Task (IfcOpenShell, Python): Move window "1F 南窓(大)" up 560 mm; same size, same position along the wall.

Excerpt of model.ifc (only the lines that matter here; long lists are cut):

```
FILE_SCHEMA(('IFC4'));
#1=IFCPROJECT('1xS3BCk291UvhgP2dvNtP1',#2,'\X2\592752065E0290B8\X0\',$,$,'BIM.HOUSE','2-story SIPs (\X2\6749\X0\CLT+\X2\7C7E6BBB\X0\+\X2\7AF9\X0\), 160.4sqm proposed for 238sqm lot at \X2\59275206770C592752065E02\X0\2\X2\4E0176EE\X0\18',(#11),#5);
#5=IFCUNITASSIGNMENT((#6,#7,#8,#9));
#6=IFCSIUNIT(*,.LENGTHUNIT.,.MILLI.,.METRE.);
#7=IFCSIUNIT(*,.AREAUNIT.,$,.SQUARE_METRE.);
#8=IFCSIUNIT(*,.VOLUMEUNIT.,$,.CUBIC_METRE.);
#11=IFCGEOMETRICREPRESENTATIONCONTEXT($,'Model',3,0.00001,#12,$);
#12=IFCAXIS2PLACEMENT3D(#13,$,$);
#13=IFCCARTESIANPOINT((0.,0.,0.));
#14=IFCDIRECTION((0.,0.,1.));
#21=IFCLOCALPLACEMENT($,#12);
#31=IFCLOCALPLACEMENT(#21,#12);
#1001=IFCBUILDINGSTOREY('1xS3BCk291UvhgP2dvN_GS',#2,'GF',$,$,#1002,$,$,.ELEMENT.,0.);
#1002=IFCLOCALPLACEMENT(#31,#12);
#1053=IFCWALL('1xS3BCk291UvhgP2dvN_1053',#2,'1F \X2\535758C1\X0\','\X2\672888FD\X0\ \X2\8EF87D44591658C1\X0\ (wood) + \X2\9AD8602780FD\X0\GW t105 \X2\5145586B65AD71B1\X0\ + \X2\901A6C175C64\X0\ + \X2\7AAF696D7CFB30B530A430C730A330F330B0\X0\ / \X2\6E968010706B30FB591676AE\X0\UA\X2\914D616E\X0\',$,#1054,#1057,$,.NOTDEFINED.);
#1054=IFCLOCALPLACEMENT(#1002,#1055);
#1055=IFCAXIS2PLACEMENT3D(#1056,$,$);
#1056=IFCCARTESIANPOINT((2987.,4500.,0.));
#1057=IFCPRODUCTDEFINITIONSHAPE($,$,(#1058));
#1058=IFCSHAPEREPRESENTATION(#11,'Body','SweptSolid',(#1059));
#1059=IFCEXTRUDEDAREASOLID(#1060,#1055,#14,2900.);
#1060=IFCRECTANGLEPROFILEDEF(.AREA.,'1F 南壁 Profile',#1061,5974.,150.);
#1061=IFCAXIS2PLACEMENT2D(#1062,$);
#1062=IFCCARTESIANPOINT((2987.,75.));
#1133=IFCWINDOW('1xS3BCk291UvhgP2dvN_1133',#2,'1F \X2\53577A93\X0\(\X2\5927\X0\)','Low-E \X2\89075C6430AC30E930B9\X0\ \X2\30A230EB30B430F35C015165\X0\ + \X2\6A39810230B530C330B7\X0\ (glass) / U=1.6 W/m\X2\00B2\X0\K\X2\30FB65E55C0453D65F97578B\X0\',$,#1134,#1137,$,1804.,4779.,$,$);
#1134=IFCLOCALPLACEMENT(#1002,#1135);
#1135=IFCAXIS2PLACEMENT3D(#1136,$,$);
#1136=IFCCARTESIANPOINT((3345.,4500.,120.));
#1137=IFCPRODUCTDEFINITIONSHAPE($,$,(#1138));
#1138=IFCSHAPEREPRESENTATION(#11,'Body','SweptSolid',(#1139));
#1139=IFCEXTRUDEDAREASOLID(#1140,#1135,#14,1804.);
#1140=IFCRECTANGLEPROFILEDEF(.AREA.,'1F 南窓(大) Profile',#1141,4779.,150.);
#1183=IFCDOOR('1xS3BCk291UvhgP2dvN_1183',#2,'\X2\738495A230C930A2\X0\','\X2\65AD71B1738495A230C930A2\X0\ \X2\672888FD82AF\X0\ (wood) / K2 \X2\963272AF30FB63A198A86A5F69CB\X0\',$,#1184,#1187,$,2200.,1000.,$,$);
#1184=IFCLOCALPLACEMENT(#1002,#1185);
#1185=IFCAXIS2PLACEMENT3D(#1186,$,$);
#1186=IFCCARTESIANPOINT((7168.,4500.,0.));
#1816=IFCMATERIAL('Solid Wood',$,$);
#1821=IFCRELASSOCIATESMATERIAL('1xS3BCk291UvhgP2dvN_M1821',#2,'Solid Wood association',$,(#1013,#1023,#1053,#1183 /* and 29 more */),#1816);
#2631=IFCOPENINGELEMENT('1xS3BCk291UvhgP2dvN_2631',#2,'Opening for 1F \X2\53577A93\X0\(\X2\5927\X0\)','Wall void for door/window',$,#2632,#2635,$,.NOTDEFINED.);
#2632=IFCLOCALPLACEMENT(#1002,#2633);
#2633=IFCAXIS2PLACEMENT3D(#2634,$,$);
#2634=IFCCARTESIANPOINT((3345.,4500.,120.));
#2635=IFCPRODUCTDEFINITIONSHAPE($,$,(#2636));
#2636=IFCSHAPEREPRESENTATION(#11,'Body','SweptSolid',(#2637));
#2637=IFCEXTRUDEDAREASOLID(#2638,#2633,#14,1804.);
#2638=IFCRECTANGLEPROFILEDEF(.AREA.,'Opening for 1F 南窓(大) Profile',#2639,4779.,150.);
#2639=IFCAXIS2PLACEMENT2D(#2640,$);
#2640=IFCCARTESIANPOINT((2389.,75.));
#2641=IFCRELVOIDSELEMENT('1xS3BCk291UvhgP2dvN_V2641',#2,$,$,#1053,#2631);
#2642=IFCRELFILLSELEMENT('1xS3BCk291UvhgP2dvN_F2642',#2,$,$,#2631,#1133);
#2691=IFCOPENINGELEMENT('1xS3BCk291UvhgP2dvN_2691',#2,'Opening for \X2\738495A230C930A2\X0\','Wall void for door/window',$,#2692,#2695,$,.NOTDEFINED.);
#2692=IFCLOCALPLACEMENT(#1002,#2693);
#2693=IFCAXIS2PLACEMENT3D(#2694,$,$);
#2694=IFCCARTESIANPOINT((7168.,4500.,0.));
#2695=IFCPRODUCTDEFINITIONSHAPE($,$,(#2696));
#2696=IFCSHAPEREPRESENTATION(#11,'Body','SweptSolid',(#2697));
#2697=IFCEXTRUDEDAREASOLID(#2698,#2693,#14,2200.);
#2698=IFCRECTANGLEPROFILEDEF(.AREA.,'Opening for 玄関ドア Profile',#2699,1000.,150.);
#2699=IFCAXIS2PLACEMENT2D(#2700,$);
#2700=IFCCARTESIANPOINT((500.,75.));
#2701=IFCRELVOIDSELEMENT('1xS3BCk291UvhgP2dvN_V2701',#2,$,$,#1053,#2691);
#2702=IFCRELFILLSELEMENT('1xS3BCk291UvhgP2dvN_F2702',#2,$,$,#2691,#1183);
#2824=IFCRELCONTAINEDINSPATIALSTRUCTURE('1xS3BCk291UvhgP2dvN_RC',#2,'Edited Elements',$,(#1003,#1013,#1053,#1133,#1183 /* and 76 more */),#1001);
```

```python
import numpy as np
import ifcopenshell
import ifcopenshell.api.geometry
import ifcopenshell.util.placement
import ifcopenshell.util.unit

model = ifcopenshell.open("model.ifc")
unit_scale = ifcopenshell.util.unit.calculate_unit_scale(model)

window = model.by_id(1133)
opening = window.FillsVoids[0].RelatingOpeningElement
dz = 560.0

shift = np.array([0.0, 0.0, dz])
# The window is not placed relative to its opening, so move both.
for product in (opening, window):
    matrix = ifcopenshell.util.placement.get_local_placement(product.ObjectPlacement)
    matrix[:3, 3] += shift
    ifcopenshell.api.geometry.edit_object_placement(model, product=product, matrix=matrix, is_si=False)

print(f"moved by {dz * unit_scale:+.3f} m")

model.write("model_updated.ifc")
```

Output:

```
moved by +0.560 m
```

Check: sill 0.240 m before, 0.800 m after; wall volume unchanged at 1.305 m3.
